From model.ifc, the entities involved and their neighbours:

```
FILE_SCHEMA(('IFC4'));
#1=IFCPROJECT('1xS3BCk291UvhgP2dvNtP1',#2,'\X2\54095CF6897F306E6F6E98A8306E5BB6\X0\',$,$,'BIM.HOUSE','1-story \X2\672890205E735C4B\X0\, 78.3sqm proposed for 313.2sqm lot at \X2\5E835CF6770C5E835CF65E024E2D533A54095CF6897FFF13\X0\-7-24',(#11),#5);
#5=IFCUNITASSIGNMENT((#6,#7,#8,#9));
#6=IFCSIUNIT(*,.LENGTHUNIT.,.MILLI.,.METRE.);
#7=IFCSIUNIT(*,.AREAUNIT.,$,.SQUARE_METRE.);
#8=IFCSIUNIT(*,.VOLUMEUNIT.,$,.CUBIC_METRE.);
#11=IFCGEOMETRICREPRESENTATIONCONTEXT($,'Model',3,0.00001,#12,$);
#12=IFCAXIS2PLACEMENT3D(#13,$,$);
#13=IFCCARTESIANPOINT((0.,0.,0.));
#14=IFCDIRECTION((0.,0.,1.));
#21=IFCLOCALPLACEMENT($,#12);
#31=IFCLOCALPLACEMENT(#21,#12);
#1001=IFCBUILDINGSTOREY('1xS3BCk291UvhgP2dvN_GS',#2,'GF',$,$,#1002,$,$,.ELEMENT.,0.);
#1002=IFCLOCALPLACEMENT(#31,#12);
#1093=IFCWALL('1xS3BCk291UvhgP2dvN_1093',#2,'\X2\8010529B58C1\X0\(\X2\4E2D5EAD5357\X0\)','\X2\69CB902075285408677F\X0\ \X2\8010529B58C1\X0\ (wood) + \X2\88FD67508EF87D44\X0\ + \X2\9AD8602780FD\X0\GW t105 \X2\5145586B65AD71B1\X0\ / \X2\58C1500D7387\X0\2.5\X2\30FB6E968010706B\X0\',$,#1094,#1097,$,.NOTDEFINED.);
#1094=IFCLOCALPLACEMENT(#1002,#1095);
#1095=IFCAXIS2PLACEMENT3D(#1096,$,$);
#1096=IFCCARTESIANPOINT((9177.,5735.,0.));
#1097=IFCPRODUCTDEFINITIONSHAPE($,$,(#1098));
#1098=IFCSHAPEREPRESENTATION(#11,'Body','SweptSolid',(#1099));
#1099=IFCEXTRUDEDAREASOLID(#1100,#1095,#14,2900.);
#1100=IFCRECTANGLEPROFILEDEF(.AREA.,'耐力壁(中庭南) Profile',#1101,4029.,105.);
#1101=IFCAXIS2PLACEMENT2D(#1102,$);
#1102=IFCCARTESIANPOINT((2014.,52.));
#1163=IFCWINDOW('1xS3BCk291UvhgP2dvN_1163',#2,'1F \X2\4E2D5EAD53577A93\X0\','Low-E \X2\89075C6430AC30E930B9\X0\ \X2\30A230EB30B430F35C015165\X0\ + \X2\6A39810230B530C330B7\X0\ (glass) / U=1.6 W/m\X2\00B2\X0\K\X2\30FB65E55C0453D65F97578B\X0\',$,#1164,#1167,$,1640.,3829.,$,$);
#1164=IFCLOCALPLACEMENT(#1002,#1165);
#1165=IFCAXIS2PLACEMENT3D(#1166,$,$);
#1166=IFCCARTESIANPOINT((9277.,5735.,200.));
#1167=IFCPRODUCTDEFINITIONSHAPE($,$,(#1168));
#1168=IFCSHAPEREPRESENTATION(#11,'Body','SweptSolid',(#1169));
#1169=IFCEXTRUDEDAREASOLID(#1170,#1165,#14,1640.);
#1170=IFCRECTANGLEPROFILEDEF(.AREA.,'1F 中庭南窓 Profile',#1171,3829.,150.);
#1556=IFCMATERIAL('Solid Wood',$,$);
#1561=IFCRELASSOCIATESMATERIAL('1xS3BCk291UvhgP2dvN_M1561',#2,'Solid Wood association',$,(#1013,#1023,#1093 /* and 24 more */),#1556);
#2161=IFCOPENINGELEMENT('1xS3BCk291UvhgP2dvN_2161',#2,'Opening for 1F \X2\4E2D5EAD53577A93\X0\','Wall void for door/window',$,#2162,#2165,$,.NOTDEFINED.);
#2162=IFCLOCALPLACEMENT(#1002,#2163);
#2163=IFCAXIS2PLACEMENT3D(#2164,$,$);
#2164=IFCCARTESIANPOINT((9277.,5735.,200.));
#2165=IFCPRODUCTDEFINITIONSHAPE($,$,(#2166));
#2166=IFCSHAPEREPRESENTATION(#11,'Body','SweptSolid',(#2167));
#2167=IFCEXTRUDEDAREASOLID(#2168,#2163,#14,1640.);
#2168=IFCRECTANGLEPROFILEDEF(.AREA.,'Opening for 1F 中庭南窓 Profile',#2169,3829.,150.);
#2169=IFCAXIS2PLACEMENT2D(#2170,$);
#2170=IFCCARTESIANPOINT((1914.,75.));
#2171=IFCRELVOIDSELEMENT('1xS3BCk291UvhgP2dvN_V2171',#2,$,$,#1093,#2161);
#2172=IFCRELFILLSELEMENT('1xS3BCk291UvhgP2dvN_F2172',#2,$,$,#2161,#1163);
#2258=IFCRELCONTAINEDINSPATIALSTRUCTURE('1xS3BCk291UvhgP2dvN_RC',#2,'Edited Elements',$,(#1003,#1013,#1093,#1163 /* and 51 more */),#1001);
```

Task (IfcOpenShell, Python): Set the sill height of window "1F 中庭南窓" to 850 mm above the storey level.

```python
import numpy as np
import ifcopenshell
import ifcopenshell.api.geometry
import ifcopenshell.geom
import ifcopenshell.util.element
import ifcopenshell.util.placement
import ifcopenshell.util.shape
import ifcopenshell.util.unit

model = ifcopenshell.open("model.ifc")
unit_scale = ifcopenshell.util.unit.calculate_unit_scale(model)

window = model.by_guid("1xS3BCk291UvhgP2dvN_1163")
opening = window.FillsVoids[0].RelatingOpeningElement
storey = ifcopenshell.util.element.get_container(window, ifc_class="IfcBuildingStorey")
level = ifcopenshell.util.placement.get_local_placement(storey.ObjectPlacement)[2, 3]

# The opening's origin need not be at the sill, so measure its lowest point.
shape = ifcopenshell.geom.create_shape(ifcopenshell.geom.settings(), opening)
bottom = ifcopenshell.util.shape.get_shape_bottom_elevation(shape, shape.geometry) / unit_scale
dz = level + 0.85 / unit_scale - bottom

shift = np.array([0.0, 0.0, dz])
# The window is not placed relative to its opening, so move both.
for product in (opening, window):
    matrix = ifcopenshell.util.placement.get_local_placement(product.ObjectPlacement)
    matrix[:3, 3] += shift
    ifcopenshell.api.geometry.edit_object_placement(model, product=product, matrix=matrix, is_si=False)

print(f"moved by {dz * unit_scale:+.3f} m")

model.write("model_updated.ifc")
```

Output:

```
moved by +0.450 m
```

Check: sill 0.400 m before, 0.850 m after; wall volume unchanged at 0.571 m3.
